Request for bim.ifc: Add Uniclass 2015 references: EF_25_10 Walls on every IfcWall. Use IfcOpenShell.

First a look at what the model holds.

```python
import ifcopenshell

model = ifcopenshell.open("bim.ifc")
print(model.schema)
print("classifications:", [c.Name for c in model.by_type("IfcClassification")])
for ifc_class in ("IfcDoor", "IfcRoof", "IfcStair", "IfcWall", "IfcWindow"):
    print(ifc_class, len(model.by_type(ifc_class)))
```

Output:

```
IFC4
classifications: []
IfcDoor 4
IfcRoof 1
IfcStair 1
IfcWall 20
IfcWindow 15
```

```python
import ifcopenshell
import ifcopenshell.api.classification

model = ifcopenshell.open("bim.ifc")

system = ifcopenshell.api.classification.add_classification(model, classification="Uniclass 2015")

codes = {
    "IfcWall": ("EF_25_10", "Walls"),
}
for ifc_class, (code, name) in codes.items():
    products = model.by_type(ifc_class)
    ifcopenshell.api.classification.add_reference(
        model, products=products, classification=system, identification=code, name=name
    )
    print(code, len(products))

model.write("bim_v2.ifc")
```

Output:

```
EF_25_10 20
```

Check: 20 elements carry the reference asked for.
